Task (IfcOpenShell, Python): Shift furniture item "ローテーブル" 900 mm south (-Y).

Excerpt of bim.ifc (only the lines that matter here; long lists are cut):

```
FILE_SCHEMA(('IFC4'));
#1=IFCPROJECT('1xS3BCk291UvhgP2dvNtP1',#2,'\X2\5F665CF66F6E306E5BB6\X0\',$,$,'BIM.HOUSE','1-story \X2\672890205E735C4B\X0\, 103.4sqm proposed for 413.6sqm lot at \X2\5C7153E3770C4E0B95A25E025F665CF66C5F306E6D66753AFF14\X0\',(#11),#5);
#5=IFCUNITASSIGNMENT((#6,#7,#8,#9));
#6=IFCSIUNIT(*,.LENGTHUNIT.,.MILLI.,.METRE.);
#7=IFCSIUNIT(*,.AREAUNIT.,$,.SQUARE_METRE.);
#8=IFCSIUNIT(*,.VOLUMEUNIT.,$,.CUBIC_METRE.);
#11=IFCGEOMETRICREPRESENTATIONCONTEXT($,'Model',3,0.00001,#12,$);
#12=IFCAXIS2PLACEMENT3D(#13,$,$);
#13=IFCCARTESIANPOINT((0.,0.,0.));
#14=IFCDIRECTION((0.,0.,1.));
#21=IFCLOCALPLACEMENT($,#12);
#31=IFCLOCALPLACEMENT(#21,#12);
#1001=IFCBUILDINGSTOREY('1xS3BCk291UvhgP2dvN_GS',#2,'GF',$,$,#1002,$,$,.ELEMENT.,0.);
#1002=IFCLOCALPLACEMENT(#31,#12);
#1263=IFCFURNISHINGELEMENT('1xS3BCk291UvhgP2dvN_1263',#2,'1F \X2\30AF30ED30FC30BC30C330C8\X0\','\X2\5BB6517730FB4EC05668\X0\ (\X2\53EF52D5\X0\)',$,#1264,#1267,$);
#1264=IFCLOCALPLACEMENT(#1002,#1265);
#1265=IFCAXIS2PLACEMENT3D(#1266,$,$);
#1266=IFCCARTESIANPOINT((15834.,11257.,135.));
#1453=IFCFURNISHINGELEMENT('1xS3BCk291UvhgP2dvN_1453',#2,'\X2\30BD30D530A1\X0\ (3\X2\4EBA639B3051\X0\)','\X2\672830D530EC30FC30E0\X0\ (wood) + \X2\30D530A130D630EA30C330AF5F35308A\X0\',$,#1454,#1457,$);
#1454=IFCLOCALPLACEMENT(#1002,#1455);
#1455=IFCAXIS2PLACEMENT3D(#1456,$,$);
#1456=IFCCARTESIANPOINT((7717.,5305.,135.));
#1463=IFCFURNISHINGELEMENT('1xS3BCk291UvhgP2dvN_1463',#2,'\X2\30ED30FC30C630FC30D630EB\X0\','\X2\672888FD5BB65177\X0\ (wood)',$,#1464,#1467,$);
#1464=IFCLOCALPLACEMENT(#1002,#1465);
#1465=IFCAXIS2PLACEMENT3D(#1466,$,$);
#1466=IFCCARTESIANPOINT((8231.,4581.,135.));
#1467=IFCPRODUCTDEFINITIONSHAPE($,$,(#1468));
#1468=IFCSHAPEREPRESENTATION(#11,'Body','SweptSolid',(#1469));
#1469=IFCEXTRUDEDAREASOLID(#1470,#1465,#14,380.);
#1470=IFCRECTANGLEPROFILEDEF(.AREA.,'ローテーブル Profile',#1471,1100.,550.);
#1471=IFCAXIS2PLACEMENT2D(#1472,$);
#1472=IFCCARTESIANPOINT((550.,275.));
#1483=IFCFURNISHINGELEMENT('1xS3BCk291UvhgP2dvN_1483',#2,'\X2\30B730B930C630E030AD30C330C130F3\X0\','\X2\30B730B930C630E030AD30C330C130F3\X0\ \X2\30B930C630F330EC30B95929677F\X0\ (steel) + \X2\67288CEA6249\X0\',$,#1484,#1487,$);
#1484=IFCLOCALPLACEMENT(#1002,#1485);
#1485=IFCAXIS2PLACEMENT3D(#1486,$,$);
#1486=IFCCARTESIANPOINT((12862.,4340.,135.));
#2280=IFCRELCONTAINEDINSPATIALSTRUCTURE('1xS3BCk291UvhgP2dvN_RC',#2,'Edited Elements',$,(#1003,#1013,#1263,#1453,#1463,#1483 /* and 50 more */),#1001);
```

```python
import ifcopenshell
import ifcopenshell.api.geometry
import ifcopenshell.util.placement

model = ifcopenshell.open("bim.ifc")

item = model.by_guid("1xS3BCk291UvhgP2dvN_1463")
matrix = ifcopenshell.util.placement.get_local_placement(item.ObjectPlacement)
matrix[1, 3] -= 900.0
ifcopenshell.api.geometry.edit_object_placement(model, product=item, matrix=matrix, is_si=False)

print(ifcopenshell.util.placement.get_local_placement(item.ObjectPlacement).round(3) + 0.0)

model.write("bim-out.ifc")
```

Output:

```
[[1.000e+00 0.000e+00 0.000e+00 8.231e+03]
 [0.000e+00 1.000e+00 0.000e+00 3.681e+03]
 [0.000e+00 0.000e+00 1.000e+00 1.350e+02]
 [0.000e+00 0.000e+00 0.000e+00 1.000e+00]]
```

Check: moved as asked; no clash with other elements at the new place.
